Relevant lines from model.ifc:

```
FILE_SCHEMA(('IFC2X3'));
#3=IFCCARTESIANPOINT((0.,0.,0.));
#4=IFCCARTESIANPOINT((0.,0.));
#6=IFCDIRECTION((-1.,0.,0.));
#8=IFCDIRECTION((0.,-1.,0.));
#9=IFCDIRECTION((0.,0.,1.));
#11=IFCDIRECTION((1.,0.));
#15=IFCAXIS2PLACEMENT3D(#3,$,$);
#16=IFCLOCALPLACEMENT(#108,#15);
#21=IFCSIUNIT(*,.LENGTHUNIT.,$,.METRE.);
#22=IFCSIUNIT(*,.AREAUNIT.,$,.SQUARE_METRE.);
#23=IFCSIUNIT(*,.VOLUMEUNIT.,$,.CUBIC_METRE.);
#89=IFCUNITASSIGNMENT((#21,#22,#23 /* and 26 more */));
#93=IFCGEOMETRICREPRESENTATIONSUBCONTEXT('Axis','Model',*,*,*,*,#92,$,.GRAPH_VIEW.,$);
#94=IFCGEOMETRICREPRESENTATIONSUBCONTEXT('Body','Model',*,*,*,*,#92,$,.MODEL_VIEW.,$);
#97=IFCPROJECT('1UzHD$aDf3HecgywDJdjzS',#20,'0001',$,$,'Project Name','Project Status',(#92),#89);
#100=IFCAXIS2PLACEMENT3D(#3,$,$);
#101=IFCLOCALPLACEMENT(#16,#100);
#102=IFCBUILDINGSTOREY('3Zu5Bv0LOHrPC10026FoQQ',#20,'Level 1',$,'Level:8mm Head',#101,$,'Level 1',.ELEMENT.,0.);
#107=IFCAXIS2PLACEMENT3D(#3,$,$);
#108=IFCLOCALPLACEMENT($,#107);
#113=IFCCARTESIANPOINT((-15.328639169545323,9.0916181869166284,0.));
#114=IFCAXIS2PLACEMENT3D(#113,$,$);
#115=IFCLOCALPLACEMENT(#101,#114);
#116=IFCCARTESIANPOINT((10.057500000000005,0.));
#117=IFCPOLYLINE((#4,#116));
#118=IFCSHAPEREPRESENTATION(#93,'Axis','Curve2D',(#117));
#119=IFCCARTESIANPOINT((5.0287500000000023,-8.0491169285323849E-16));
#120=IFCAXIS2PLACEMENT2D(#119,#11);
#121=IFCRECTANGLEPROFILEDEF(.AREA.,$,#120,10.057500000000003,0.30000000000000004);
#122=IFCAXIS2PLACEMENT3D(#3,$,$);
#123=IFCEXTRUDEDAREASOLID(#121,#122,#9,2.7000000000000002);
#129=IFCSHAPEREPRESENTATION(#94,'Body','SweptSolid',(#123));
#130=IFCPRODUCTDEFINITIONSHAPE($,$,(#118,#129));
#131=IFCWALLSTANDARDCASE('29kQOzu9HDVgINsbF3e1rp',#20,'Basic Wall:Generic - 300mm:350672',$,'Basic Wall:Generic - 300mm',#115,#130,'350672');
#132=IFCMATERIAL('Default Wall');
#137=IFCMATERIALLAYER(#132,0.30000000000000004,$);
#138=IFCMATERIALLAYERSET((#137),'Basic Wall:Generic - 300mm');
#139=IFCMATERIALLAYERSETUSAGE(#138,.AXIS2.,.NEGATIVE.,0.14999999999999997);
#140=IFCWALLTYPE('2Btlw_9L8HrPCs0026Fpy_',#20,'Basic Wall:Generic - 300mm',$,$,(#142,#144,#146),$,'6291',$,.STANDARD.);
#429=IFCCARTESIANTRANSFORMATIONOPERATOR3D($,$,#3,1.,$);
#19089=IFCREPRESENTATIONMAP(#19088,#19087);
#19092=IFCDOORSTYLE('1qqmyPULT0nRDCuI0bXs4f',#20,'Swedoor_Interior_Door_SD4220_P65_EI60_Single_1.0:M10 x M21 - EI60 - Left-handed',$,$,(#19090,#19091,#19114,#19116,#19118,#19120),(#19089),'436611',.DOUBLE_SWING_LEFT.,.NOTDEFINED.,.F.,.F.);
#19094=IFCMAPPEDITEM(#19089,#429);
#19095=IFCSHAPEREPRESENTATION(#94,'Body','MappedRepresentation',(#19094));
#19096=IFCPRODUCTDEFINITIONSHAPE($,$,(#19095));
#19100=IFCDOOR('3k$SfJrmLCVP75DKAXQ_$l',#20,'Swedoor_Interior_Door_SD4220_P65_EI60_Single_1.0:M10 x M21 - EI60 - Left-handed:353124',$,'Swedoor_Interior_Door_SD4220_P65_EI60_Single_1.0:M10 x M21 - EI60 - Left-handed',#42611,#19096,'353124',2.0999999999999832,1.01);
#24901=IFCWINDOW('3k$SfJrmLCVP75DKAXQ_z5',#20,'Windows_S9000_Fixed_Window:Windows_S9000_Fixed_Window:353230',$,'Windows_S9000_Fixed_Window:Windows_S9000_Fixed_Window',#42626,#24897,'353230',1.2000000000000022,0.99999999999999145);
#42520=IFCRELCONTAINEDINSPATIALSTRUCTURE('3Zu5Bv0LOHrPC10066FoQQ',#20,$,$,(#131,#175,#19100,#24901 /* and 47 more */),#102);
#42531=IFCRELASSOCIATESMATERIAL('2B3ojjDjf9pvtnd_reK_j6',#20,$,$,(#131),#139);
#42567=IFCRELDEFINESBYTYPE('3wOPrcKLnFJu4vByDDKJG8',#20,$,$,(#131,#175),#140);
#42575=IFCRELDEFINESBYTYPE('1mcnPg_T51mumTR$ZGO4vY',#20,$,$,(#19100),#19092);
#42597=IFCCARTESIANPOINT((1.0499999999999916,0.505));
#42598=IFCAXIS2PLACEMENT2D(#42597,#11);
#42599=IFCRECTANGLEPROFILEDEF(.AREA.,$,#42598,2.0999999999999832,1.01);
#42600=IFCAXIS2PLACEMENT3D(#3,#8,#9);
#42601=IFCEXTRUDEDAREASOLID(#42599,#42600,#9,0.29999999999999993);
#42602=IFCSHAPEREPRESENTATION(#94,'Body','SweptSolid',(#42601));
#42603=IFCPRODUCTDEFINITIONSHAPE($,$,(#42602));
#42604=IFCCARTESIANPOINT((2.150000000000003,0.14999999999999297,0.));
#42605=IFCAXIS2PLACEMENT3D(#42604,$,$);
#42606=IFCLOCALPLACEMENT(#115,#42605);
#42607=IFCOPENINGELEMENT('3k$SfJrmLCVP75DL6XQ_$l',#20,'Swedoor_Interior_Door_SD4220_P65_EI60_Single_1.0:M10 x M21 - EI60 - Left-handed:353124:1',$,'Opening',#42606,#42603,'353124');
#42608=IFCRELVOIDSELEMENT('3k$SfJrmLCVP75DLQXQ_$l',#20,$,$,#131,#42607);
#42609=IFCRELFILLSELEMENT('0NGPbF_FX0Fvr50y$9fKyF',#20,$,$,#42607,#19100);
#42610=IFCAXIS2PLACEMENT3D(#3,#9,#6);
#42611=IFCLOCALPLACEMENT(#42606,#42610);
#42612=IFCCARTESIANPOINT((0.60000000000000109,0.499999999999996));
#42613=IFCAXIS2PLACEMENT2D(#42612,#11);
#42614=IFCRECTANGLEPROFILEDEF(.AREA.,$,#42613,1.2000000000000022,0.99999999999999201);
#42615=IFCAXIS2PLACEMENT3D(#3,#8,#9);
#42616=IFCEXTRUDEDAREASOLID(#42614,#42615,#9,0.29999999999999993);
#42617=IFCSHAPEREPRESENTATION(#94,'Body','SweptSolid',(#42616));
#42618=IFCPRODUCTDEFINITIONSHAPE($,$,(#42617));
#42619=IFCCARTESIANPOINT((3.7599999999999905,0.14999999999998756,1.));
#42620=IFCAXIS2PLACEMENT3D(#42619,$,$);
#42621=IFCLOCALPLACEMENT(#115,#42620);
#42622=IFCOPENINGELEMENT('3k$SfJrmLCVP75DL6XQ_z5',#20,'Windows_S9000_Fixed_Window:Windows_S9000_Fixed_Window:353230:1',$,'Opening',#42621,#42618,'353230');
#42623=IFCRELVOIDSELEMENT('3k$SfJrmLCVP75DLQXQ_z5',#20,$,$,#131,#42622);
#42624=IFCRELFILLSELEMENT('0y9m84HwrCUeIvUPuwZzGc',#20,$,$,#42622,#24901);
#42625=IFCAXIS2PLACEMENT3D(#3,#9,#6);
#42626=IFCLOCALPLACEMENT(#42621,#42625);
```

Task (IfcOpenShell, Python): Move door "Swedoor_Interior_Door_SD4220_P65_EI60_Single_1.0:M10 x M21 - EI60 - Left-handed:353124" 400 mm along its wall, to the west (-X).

```python
import ifcopenshell
import ifcopenshell.api.geometry
import ifcopenshell.util.placement
import ifcopenshell.util.unit

model = ifcopenshell.open("model.ifc")
unit_scale = ifcopenshell.util.unit.calculate_unit_scale(model)

door = model.by_id(19100)
opening = door.FillsVoids[0].RelatingOpeningElement
wall = opening.VoidsElements[0].RelatingBuildingElement

wall_matrix = ifcopenshell.util.placement.get_local_placement(wall.ObjectPlacement)
shift = wall_matrix[:3, 0] * -0.4 / unit_scale
before = ifcopenshell.util.placement.get_local_placement(door.ObjectPlacement)[:3, 3].copy()

# The door is placed relative to its opening, so it follows when the opening moves.
matrix = ifcopenshell.util.placement.get_local_placement(opening.ObjectPlacement)
matrix[:3, 3] += shift
ifcopenshell.api.geometry.edit_object_placement(
    model, product=opening, matrix=matrix, is_si=False, should_transform_children=True
)

after = ifcopenshell.util.placement.get_local_placement(door.ObjectPlacement)[:3, 3]
print("door moved by", (after - before).round(3) + 0.0)

model.write("model_edited.ifc")
```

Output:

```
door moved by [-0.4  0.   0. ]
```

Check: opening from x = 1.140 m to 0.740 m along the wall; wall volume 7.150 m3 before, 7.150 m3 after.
